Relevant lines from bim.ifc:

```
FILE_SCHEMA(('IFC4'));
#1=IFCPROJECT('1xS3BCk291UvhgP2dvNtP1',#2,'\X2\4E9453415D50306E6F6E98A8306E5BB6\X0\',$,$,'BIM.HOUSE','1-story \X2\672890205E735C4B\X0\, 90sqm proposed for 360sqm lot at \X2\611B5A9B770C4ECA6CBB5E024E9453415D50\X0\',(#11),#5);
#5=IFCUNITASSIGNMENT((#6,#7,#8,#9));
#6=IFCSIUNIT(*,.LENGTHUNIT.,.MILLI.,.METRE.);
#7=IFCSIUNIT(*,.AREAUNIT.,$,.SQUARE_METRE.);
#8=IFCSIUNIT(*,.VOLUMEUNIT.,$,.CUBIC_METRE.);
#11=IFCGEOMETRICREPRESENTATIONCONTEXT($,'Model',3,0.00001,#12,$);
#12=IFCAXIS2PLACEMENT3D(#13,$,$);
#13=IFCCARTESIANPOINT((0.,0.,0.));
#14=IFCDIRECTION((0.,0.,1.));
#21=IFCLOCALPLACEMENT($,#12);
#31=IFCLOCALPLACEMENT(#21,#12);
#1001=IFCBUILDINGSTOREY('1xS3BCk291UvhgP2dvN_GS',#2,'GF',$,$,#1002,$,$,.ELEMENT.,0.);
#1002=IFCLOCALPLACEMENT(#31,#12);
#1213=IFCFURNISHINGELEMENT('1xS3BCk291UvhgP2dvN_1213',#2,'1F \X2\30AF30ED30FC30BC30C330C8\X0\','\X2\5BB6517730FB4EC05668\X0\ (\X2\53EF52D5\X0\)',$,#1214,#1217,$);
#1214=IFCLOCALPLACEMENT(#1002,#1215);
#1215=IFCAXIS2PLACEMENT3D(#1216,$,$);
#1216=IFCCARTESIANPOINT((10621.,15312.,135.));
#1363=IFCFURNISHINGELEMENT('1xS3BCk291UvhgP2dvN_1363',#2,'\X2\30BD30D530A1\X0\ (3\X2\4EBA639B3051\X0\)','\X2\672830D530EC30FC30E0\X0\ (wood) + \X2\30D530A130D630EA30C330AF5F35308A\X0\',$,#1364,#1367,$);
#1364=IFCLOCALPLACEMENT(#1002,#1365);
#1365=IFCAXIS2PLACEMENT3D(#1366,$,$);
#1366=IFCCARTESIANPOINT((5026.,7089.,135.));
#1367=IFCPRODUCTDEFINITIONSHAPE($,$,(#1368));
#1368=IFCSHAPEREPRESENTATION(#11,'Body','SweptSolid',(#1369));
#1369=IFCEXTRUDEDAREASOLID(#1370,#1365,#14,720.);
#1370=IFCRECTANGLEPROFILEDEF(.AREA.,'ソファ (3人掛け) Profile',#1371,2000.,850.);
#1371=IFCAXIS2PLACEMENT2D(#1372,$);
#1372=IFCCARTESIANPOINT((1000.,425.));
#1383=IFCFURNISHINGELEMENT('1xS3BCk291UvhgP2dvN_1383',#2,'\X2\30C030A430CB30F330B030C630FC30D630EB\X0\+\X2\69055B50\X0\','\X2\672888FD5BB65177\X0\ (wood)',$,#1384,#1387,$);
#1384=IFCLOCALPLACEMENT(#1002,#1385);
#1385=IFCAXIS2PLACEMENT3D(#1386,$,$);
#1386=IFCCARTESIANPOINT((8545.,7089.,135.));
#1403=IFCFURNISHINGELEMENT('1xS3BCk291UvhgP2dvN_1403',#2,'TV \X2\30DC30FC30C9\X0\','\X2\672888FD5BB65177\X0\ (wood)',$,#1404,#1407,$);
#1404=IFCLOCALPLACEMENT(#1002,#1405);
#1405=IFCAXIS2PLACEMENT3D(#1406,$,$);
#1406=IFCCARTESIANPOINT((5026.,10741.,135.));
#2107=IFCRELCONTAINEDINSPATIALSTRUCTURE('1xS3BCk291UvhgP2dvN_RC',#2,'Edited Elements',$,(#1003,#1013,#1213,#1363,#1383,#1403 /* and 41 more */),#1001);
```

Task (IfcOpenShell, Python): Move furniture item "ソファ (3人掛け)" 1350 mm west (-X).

```python
import ifcopenshell
import ifcopenshell.api.geometry
import ifcopenshell.util.placement
import ifcopenshell.util.unit

model = ifcopenshell.open("bim.ifc")
unit_scale = ifcopenshell.util.unit.calculate_unit_scale(model)

item = model.by_id(1363)
matrix = ifcopenshell.util.placement.get_local_placement(item.ObjectPlacement)
matrix[0, 3] -= 1.35 / unit_scale
ifcopenshell.api.geometry.edit_object_placement(model, product=item, matrix=matrix, is_si=False)

print(ifcopenshell.util.placement.get_local_placement(item.ObjectPlacement).round(3) + 0.0)

model.write("bim_rev.ifc")
```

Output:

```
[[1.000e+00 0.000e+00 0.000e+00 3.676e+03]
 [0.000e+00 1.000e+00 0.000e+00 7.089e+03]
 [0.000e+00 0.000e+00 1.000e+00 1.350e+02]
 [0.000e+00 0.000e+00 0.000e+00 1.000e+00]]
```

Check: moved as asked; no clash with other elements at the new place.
